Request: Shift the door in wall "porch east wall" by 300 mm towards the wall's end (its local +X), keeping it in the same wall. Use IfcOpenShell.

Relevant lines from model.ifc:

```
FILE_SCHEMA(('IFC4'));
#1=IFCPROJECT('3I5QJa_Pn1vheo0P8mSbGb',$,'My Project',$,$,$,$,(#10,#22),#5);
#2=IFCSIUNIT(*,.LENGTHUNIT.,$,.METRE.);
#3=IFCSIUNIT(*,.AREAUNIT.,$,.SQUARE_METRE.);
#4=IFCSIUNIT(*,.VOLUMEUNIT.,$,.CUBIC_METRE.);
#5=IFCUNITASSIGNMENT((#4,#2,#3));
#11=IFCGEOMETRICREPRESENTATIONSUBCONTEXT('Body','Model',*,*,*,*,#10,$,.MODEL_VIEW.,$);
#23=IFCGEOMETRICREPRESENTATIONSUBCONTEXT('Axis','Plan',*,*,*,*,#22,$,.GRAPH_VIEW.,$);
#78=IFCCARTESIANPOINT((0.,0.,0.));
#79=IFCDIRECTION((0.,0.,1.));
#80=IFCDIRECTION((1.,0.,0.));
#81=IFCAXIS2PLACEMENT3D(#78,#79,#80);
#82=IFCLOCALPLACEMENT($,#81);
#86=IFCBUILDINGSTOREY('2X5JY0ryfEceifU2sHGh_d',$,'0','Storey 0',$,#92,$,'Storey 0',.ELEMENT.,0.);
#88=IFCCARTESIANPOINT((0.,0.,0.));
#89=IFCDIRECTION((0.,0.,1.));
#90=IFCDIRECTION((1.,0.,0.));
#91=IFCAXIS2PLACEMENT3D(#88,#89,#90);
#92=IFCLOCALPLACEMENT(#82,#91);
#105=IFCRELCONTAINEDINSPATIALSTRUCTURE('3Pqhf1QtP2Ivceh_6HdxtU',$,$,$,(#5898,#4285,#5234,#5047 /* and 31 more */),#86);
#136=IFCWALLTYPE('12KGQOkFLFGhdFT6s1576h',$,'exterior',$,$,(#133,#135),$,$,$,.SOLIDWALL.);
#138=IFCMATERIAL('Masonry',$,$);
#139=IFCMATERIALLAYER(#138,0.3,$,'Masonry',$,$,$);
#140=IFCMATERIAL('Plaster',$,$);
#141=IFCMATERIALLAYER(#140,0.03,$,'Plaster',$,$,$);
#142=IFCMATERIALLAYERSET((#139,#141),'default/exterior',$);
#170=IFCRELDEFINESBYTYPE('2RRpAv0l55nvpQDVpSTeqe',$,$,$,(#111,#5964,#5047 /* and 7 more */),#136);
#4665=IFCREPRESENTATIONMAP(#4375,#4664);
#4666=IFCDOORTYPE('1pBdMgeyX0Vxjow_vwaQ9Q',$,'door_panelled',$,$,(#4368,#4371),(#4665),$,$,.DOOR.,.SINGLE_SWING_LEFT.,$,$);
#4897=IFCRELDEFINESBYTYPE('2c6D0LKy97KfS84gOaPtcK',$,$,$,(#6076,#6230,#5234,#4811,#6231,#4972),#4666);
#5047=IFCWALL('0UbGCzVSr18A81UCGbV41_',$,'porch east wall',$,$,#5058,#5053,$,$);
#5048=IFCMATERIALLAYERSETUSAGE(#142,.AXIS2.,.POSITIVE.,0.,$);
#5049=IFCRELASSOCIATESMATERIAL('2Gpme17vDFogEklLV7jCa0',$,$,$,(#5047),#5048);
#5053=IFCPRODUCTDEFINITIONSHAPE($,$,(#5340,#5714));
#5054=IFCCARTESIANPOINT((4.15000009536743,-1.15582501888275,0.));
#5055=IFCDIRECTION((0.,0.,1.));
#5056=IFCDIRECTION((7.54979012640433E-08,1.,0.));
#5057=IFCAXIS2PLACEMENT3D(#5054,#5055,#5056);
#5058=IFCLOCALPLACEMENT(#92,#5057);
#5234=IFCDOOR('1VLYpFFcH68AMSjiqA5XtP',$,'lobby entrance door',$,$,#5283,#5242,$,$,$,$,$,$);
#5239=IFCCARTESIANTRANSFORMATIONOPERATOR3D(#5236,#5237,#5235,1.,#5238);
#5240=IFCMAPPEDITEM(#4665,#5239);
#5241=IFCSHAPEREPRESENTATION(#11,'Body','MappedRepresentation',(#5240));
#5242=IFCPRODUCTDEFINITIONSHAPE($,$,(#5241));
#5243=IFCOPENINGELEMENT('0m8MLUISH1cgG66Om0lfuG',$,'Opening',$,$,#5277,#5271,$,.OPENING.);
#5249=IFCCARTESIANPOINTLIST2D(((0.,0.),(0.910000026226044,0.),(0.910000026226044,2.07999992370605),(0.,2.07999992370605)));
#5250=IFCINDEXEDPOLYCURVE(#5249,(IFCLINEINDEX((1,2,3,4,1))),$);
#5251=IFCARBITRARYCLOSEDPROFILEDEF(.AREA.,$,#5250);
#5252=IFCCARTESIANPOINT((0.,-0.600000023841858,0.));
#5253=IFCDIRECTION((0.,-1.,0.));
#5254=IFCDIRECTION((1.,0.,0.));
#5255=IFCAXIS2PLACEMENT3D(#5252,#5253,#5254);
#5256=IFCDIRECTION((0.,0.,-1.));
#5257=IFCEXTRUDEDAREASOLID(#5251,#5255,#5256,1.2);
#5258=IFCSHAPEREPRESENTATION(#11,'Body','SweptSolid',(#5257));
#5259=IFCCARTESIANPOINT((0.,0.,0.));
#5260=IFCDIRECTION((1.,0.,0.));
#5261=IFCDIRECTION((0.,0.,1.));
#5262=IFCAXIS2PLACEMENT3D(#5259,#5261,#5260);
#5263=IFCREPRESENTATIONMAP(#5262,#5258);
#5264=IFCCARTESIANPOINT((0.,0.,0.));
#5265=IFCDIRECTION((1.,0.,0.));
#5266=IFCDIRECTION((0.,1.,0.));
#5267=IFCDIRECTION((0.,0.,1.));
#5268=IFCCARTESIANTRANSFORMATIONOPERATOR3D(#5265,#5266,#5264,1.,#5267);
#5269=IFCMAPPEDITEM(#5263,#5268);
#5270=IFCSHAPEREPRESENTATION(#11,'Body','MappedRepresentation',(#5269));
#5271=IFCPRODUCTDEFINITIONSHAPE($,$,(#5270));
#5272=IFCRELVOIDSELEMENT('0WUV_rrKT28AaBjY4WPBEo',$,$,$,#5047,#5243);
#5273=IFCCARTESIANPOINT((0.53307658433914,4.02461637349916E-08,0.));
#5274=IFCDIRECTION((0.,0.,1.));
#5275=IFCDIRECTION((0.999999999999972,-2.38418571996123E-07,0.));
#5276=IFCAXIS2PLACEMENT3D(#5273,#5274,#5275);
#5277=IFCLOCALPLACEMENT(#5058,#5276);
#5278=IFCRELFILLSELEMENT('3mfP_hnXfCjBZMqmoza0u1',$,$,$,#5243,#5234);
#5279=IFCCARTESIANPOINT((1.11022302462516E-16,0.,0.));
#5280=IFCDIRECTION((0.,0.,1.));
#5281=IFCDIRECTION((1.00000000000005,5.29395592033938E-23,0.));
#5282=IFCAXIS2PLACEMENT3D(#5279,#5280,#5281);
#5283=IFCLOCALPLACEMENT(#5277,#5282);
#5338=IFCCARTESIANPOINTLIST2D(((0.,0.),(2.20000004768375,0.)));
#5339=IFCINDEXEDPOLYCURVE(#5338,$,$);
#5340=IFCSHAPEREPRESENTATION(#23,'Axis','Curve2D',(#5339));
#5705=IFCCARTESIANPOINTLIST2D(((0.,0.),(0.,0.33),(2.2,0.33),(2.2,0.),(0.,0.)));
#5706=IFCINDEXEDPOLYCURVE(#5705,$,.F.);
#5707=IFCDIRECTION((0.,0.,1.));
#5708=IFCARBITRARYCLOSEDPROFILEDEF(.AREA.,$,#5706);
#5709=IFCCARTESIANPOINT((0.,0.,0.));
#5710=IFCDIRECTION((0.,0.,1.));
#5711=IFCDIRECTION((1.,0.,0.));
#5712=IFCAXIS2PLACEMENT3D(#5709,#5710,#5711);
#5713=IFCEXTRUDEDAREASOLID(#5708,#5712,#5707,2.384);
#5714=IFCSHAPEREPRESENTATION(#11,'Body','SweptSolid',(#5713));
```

```python
import ifcopenshell
import ifcopenshell.api.geometry
import ifcopenshell.util.placement
import ifcopenshell.util.unit

model = ifcopenshell.open("model.ifc")
unit_scale = ifcopenshell.util.unit.calculate_unit_scale(model)

door = model.by_guid("1VLYpFFcH68AMSjiqA5XtP")
opening = door.FillsVoids[0].RelatingOpeningElement
wall = opening.VoidsElements[0].RelatingBuildingElement

wall_matrix = ifcopenshell.util.placement.get_local_placement(wall.ObjectPlacement)
shift = wall_matrix[:3, 0] * 0.3 / unit_scale
before = ifcopenshell.util.placement.get_local_placement(door.ObjectPlacement)[:3, 3].copy()

# The door is placed relative to its opening, so it follows when the opening moves.
matrix = ifcopenshell.util.placement.get_local_placement(opening.ObjectPlacement)
matrix[:3, 3] += shift
ifcopenshell.api.geometry.edit_object_placement(
    model, product=opening, matrix=matrix, is_si=False, should_transform_children=True
)

after = ifcopenshell.util.placement.get_local_placement(door.ObjectPlacement)[:3, 3]
print("door moved by", (after - before).round(3) + 0.0)

model.write("model_v2.ifc")
```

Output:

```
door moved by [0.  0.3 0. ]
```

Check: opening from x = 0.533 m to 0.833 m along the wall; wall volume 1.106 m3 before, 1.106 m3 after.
